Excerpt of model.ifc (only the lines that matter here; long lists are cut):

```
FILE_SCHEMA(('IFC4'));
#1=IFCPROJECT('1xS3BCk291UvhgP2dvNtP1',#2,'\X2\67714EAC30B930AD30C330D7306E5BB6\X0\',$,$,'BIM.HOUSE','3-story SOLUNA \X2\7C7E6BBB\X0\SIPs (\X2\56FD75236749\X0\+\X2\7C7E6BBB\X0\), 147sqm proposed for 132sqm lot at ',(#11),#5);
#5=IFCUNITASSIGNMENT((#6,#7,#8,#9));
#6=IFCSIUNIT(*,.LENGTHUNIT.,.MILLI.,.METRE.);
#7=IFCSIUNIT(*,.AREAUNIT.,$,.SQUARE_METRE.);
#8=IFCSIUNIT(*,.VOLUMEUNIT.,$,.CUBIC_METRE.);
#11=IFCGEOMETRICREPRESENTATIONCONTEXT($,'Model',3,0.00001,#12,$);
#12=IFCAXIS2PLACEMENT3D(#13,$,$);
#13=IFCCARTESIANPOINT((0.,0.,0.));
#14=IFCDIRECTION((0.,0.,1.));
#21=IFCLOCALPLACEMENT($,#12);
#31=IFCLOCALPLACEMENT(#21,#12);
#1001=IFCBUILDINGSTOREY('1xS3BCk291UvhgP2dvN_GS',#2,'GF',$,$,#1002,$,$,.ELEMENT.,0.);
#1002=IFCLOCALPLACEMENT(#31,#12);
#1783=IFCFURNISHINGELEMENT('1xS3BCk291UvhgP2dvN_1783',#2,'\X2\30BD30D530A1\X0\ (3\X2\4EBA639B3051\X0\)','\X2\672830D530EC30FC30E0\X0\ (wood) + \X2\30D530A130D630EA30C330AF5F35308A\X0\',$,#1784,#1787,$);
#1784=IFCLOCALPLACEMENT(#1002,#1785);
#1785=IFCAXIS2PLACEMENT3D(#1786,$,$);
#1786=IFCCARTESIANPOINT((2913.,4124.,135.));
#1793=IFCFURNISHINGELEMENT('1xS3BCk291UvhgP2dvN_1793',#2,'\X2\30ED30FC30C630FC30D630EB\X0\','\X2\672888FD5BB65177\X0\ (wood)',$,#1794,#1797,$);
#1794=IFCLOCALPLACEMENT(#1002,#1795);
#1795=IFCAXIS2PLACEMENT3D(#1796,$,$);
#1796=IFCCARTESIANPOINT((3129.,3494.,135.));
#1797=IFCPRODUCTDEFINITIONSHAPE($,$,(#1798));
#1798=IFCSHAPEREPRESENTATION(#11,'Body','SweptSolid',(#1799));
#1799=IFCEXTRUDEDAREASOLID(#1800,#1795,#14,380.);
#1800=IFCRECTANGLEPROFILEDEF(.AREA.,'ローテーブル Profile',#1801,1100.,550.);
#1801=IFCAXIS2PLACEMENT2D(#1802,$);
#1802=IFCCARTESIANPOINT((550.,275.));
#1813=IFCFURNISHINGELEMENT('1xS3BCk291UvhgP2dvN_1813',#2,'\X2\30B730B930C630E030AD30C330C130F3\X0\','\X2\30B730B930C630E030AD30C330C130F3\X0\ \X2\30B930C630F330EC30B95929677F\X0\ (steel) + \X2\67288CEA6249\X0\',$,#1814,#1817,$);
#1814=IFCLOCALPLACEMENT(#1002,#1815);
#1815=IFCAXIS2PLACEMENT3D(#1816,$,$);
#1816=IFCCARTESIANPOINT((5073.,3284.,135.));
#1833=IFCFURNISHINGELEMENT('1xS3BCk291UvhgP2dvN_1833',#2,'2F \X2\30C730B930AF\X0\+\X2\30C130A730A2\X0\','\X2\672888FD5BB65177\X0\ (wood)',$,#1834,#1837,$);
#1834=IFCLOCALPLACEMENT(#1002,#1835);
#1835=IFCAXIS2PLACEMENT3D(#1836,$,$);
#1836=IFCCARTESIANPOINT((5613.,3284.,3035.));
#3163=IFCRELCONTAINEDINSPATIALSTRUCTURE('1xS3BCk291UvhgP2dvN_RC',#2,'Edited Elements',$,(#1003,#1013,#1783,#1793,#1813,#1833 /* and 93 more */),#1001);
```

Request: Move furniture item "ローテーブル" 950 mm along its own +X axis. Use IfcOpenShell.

```python
import ifcopenshell
import ifcopenshell.api.geometry
import ifcopenshell.util.placement

model = ifcopenshell.open("model.ifc")

item = model.by_guid("1xS3BCk291UvhgP2dvN_1793")
matrix = ifcopenshell.util.placement.get_local_placement(item.ObjectPlacement)
matrix[:3, 3] += matrix[:3, 0] * 950.0
ifcopenshell.api.geometry.edit_object_placement(model, product=item, matrix=matrix, is_si=False)

print(ifcopenshell.util.placement.get_local_placement(item.ObjectPlacement).round(3) + 0.0)

model.write("model_rev.ifc")
```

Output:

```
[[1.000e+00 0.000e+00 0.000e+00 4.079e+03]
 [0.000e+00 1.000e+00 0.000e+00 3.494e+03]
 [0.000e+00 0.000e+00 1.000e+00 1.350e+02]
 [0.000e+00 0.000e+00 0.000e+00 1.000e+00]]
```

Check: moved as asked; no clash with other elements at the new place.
